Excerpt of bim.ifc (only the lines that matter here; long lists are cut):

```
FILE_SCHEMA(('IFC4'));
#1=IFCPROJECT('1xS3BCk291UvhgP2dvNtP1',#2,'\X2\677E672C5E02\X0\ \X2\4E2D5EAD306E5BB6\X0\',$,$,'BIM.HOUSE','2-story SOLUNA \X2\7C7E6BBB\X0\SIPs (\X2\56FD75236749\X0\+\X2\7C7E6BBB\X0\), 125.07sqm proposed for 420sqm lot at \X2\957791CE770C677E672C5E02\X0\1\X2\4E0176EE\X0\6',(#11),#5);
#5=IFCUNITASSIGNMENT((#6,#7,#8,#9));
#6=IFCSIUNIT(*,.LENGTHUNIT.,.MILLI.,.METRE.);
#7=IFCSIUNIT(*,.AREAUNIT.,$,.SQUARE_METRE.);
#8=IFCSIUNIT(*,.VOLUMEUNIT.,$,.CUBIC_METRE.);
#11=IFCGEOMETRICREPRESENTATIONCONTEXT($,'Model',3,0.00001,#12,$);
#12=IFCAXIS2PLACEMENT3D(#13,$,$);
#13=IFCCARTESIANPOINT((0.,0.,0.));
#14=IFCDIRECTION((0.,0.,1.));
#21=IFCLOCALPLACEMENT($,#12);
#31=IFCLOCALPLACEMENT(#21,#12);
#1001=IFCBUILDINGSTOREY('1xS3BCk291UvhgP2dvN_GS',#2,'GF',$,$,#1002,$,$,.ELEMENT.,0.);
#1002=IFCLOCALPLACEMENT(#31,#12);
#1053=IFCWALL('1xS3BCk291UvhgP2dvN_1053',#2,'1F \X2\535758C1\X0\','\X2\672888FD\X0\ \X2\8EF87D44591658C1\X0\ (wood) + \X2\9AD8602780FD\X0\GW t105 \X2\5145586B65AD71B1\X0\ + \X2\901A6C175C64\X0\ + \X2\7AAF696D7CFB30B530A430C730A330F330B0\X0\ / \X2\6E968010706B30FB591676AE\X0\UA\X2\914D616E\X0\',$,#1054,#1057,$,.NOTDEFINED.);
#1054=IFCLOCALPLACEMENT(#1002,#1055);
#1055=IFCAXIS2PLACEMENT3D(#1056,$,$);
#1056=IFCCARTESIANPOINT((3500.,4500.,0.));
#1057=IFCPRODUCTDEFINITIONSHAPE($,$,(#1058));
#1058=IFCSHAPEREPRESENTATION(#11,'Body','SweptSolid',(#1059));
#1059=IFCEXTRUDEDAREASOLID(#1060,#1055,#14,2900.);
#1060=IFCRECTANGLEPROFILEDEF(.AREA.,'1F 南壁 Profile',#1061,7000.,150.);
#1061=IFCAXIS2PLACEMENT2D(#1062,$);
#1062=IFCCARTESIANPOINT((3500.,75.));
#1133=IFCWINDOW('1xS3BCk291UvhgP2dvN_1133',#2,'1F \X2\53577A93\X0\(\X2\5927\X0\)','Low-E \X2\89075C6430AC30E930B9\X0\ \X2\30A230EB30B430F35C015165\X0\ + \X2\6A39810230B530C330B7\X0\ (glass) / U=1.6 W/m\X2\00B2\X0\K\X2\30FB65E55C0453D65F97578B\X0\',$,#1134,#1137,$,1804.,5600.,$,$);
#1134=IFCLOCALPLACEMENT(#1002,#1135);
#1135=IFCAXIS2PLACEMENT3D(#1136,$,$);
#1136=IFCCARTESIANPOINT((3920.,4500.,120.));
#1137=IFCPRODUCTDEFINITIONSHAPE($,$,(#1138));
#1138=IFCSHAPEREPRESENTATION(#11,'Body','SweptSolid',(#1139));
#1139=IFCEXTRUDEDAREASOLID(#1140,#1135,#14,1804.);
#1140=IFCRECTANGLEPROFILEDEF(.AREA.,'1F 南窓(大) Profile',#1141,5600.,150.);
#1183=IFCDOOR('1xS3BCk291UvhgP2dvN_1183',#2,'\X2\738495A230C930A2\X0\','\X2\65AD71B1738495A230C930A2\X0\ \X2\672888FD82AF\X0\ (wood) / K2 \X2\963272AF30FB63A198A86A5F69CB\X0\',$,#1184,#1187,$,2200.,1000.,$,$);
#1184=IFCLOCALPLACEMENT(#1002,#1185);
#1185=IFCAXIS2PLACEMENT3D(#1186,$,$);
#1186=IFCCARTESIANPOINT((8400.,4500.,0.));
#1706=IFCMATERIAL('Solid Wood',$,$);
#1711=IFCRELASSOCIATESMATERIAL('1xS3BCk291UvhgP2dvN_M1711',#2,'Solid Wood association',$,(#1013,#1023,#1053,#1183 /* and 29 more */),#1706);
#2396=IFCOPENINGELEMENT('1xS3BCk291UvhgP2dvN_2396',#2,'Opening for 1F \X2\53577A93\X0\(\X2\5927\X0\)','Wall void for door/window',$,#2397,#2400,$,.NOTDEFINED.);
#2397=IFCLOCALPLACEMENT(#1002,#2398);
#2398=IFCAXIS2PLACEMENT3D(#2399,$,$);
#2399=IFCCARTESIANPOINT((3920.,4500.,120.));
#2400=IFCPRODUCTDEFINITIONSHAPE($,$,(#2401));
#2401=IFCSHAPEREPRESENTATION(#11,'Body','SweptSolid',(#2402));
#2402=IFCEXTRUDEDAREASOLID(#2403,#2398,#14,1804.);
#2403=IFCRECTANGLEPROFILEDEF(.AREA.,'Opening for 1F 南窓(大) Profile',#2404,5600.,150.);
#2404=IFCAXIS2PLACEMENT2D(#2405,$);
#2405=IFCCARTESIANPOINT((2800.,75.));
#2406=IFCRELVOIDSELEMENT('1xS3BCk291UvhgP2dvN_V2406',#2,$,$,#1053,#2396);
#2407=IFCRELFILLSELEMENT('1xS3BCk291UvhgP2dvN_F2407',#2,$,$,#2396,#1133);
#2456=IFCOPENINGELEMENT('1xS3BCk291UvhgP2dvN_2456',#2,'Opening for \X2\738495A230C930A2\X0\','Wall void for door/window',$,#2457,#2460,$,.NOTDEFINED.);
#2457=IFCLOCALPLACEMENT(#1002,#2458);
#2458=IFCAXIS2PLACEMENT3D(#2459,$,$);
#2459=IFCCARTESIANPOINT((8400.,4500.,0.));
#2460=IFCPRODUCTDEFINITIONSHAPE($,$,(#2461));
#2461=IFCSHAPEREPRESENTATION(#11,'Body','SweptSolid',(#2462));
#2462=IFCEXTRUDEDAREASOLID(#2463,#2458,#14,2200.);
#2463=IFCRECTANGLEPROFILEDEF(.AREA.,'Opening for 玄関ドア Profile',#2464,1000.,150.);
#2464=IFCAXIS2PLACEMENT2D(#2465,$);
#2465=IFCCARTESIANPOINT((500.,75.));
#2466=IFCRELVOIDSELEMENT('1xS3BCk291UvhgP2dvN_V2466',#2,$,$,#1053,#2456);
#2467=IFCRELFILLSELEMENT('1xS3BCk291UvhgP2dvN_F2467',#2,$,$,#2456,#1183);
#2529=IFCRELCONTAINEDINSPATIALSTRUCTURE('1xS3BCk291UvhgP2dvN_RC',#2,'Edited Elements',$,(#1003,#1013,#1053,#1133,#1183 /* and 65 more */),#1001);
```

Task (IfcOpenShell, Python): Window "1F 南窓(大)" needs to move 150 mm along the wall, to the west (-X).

```python
import ifcopenshell
import ifcopenshell.api.geometry
import ifcopenshell.util.placement
import ifcopenshell.util.unit

model = ifcopenshell.open("bim.ifc")
unit_scale = ifcopenshell.util.unit.calculate_unit_scale(model)

window = model.by_guid("1xS3BCk291UvhgP2dvN_1133")
opening = window.FillsVoids[0].RelatingOpeningElement
wall = opening.VoidsElements[0].RelatingBuildingElement

wall_matrix = ifcopenshell.util.placement.get_local_placement(wall.ObjectPlacement)
shift = wall_matrix[:3, 0] * -0.15 / unit_scale
before = ifcopenshell.util.placement.get_local_placement(window.ObjectPlacement)[:3, 3].copy()

# The window is not placed relative to its opening, so move both.
for product in (opening, window):
    matrix = ifcopenshell.util.placement.get_local_placement(product.ObjectPlacement)
    matrix[:3, 3] += shift
    ifcopenshell.api.geometry.edit_object_placement(model, product=product, matrix=matrix, is_si=False)

after = ifcopenshell.util.placement.get_local_placement(window.ObjectPlacement)[:3, 3]
print("window moved by", (after - before).round(3) + 0.0)

model.write("bim_v2.ifc")
```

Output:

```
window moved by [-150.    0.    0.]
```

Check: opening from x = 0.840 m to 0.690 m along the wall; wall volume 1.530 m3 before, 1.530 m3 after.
